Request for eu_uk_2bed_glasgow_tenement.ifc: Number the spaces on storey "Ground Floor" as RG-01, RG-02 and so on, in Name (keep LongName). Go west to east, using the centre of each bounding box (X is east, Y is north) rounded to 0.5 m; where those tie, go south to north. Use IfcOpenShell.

First a look at what the model holds.

```python
import ifcopenshell
import ifcopenshell.util.element
import ifcopenshell.util.placement

model = ifcopenshell.open("eu_uk_2bed_glasgow_tenement.ifc")
print(model.schema)
storey = next(s for s in model.by_type("IfcBuildingStorey") if s.Name == "Ground Floor")
spaces = [e for e in ifcopenshell.util.element.get_decomposition(storey) if e.is_a("IfcSpace")]
for e in sorted(spaces, key=lambda e: e.id()):
    origin = ifcopenshell.util.placement.get_local_placement(e.ObjectPlacement)[:3, 3]
    print(e.id(), e.Name, e.LongName, origin.round(2) + 0.0, sep=" | ")
```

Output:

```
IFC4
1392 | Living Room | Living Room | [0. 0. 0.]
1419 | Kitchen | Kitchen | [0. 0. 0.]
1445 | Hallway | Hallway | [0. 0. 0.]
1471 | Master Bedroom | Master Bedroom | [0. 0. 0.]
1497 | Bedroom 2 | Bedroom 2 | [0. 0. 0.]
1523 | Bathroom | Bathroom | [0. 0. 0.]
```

```python
import ifcopenshell
import ifcopenshell.geom
import ifcopenshell.util.element
import ifcopenshell.util.shape

model = ifcopenshell.open("eu_uk_2bed_glasgow_tenement.ifc")
settings = ifcopenshell.geom.settings()
settings.set("use-world-coords", True)


def centre(element):
    shape = ifcopenshell.geom.create_shape(settings, element)
    return ifcopenshell.util.shape.get_bbox_centroid(shape.geometry)


storey = next(s for s in model.by_type("IfcBuildingStorey") if s.Name == "Ground Floor")
spaces = [e for e in ifcopenshell.util.element.get_decomposition(storey) if e.is_a("IfcSpace")]

# Insertion points can sit at a corner or the storey origin, so sort by the geometry (in metres).
centres = {e: centre(e) for e in spaces}
spaces.sort(key=lambda e: (round(centres[e][0] / 0.5), centres[e][1]))

for i, e in enumerate(spaces, start=1):
    number = f"RG-{i:02d}"
    e.Name = number
    print(e.id(), number)

model.write("eu_uk_2bed_glasgow_tenement_edited.ifc")
```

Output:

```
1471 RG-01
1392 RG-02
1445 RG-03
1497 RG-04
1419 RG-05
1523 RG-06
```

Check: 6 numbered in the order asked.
